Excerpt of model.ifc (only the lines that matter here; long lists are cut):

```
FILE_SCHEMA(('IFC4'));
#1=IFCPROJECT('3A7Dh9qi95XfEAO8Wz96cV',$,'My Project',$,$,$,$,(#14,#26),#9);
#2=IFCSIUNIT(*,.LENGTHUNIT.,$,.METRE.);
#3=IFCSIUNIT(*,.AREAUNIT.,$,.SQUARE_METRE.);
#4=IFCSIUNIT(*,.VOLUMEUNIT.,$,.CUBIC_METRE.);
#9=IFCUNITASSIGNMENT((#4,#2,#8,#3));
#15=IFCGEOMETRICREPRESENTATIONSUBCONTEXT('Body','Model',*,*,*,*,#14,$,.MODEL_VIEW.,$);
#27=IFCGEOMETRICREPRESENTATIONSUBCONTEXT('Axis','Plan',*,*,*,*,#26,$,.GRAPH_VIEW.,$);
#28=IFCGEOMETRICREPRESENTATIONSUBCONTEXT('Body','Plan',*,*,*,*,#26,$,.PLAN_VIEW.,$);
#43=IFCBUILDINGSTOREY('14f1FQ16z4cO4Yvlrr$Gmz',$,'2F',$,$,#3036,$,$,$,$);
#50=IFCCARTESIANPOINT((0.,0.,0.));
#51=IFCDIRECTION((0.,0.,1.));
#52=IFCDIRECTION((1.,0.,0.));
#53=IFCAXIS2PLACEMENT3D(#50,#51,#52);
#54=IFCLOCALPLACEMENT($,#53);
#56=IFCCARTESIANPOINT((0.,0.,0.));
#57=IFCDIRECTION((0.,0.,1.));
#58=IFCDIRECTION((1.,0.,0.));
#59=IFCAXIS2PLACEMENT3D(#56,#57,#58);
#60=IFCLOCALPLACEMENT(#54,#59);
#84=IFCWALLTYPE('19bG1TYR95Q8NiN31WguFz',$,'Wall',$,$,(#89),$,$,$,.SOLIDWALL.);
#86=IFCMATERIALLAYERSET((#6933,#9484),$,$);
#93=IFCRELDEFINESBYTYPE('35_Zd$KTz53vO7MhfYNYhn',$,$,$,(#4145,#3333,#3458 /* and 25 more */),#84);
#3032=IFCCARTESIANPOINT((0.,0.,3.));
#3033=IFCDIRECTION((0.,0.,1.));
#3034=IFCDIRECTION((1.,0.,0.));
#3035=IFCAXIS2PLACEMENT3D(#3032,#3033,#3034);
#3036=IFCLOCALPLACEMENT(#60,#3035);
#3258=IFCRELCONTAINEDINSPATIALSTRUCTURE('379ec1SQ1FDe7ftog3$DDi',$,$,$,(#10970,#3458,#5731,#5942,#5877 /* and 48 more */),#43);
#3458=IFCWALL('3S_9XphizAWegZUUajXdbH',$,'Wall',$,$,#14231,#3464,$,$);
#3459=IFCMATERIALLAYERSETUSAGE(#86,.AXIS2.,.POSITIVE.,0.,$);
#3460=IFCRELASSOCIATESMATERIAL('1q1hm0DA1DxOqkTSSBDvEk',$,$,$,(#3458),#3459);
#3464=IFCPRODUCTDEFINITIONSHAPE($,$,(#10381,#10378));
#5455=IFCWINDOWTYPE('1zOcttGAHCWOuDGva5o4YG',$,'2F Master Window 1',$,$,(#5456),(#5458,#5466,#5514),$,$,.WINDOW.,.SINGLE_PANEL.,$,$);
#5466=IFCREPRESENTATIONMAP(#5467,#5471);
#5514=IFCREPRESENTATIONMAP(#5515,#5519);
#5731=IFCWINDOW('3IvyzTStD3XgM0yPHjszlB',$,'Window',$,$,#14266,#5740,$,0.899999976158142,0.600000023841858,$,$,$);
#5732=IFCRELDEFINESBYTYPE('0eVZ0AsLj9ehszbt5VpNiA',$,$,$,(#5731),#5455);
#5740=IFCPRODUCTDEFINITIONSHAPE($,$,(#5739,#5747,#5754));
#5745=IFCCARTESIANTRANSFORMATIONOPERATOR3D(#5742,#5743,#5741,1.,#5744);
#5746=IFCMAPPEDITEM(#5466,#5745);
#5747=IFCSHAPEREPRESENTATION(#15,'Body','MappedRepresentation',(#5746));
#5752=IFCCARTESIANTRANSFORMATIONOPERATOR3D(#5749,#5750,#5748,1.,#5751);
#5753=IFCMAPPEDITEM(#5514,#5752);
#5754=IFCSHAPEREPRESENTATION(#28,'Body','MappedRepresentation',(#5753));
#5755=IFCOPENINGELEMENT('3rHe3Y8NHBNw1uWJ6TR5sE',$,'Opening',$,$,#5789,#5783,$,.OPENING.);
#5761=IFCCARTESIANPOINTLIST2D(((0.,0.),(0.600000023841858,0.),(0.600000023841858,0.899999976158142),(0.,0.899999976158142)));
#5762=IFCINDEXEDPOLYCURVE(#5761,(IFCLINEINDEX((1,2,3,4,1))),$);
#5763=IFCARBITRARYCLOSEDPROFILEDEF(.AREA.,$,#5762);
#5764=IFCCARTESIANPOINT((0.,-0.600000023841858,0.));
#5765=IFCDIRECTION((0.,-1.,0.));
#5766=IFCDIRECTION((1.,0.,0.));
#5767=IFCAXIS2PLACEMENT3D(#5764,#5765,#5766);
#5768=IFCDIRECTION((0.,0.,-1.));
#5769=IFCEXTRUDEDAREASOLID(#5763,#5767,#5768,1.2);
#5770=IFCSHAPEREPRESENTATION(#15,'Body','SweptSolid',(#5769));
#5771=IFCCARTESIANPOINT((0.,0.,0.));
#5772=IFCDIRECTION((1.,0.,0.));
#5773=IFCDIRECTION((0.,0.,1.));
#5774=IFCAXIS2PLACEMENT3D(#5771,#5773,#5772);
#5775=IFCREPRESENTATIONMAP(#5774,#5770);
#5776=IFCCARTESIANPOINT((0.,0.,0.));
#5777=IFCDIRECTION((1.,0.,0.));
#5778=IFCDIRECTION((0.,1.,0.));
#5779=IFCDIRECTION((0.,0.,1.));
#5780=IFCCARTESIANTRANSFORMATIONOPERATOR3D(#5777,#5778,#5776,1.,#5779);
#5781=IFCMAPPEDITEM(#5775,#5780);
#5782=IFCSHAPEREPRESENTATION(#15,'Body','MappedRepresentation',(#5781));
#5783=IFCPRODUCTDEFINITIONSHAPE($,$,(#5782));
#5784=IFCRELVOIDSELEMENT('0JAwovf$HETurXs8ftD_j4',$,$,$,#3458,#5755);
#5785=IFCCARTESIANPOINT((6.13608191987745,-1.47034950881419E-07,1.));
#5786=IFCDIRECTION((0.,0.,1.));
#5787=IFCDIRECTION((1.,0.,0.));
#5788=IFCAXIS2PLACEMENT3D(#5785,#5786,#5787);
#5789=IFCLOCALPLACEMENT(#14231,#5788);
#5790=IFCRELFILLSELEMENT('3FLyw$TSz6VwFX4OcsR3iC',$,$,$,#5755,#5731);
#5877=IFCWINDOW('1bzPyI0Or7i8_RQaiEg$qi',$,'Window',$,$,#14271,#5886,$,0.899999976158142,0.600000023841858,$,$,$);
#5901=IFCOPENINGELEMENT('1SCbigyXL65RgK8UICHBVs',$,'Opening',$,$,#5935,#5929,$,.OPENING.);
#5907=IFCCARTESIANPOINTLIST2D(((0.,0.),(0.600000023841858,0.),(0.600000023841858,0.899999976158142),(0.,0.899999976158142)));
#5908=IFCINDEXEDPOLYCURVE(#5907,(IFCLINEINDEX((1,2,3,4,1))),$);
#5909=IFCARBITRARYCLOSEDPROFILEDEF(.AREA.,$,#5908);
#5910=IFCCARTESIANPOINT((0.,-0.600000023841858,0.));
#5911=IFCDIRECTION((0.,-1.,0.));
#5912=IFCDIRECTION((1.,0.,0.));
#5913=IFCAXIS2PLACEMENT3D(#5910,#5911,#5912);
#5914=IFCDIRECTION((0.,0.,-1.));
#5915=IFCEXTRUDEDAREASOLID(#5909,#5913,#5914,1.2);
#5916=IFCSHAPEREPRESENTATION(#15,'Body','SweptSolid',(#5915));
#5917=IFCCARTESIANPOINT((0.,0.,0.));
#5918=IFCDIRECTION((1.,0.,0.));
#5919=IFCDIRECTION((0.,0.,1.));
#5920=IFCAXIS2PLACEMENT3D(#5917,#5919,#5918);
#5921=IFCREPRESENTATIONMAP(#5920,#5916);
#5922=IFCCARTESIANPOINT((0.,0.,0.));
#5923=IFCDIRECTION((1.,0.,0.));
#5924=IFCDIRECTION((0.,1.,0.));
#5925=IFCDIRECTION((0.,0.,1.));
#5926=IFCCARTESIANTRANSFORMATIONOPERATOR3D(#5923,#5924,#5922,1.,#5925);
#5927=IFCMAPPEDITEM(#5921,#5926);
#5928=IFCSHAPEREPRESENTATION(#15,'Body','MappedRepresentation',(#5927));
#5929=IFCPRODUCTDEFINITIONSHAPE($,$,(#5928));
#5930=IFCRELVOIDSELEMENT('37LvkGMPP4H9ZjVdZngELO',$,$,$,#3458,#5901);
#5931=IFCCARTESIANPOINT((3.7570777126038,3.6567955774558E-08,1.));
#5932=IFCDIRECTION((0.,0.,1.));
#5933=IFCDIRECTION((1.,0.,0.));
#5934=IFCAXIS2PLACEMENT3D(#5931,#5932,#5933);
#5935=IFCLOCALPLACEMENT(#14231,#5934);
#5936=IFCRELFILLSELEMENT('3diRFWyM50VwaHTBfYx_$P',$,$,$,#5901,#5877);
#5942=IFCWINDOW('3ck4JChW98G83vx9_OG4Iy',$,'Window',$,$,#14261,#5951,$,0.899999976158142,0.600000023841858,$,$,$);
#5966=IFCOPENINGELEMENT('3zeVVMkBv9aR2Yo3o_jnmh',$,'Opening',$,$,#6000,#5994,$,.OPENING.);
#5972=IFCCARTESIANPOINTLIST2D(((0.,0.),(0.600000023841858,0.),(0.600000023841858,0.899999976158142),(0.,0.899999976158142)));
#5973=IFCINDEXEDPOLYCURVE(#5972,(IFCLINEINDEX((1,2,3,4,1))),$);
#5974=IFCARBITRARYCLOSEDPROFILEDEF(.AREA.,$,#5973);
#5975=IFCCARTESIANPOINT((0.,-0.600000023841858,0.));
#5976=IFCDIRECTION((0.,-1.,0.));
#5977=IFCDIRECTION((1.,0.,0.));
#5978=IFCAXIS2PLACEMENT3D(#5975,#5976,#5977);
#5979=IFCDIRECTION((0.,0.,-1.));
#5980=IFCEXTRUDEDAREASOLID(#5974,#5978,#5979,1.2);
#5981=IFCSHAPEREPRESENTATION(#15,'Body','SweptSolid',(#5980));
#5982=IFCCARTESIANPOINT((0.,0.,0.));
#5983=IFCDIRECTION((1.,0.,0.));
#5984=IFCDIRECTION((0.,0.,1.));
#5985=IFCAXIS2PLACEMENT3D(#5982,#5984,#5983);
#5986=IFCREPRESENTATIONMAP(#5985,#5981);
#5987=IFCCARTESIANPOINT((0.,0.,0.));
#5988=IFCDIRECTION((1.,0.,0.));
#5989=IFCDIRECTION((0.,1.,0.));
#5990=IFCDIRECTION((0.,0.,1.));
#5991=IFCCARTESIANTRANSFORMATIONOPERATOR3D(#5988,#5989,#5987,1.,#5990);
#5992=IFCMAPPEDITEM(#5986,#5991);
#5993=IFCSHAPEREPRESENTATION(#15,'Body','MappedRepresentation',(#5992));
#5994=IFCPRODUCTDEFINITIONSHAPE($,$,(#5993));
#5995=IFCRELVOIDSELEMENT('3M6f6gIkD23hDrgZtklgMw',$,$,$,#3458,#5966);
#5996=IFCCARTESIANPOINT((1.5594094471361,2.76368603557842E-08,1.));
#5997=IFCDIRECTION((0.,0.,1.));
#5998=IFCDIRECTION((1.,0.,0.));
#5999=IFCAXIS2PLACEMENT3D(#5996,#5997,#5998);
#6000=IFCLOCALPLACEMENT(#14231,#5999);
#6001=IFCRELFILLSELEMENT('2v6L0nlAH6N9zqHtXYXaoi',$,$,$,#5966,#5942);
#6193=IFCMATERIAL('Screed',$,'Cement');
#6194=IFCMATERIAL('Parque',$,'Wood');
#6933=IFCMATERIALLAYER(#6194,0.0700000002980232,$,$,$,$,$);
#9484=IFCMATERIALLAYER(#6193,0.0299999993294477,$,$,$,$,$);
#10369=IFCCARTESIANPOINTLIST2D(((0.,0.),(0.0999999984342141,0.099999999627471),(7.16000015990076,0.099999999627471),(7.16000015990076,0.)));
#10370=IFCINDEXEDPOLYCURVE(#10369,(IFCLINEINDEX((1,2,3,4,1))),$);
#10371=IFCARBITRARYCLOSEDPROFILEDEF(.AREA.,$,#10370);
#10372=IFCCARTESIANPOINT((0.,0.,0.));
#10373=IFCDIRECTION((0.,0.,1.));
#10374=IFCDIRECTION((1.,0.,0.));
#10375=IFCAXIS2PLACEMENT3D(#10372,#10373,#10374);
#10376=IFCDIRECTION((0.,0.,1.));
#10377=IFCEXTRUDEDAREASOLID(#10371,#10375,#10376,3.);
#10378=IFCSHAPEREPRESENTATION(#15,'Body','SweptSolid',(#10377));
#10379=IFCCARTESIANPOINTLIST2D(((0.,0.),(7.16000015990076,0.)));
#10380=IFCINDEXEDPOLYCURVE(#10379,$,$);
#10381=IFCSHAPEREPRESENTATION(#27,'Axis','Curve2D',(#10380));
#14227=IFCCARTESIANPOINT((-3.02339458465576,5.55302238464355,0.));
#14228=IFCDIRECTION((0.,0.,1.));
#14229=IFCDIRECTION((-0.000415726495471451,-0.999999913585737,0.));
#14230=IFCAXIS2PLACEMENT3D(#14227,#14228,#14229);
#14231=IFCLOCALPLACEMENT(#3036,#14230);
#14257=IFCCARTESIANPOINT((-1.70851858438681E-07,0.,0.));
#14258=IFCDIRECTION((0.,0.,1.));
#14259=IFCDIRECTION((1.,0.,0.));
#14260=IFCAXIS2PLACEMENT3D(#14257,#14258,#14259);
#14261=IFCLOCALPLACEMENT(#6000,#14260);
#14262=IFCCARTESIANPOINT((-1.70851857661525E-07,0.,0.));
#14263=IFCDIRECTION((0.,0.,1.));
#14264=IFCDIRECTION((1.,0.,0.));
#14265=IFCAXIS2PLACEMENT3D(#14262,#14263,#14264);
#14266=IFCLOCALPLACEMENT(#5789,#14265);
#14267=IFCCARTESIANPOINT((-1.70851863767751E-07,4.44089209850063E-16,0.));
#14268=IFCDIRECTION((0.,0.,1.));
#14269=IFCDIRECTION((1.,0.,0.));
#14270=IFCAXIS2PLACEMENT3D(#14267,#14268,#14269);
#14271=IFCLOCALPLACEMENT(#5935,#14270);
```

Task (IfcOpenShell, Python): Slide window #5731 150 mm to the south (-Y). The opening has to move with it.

```python
import ifcopenshell
import ifcopenshell.api.geometry
import ifcopenshell.util.placement
import ifcopenshell.util.unit

model = ifcopenshell.open("model.ifc")
unit_scale = ifcopenshell.util.unit.calculate_unit_scale(model)

window = model.by_guid("3IvyzTStD3XgM0yPHjszlB")
opening = window.FillsVoids[0].RelatingOpeningElement
wall = opening.VoidsElements[0].RelatingBuildingElement

wall_matrix = ifcopenshell.util.placement.get_local_placement(wall.ObjectPlacement)
shift = wall_matrix[:3, 0] * 0.15 / unit_scale
before = ifcopenshell.util.placement.get_local_placement(window.ObjectPlacement)[:3, 3].copy()

# The window is placed relative to its opening, so it follows when the opening moves.
matrix = ifcopenshell.util.placement.get_local_placement(opening.ObjectPlacement)
matrix[:3, 3] += shift
ifcopenshell.api.geometry.edit_object_placement(
    model, product=opening, matrix=matrix, is_si=False, should_transform_children=True
)

after = ifcopenshell.util.placement.get_local_placement(window.ObjectPlacement)[:3, 3]
print("window moved by", (after - before).round(3) + 0.0)

model.write("model-out.ifc")
```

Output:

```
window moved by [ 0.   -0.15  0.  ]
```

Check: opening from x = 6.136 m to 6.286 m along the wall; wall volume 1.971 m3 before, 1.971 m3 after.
